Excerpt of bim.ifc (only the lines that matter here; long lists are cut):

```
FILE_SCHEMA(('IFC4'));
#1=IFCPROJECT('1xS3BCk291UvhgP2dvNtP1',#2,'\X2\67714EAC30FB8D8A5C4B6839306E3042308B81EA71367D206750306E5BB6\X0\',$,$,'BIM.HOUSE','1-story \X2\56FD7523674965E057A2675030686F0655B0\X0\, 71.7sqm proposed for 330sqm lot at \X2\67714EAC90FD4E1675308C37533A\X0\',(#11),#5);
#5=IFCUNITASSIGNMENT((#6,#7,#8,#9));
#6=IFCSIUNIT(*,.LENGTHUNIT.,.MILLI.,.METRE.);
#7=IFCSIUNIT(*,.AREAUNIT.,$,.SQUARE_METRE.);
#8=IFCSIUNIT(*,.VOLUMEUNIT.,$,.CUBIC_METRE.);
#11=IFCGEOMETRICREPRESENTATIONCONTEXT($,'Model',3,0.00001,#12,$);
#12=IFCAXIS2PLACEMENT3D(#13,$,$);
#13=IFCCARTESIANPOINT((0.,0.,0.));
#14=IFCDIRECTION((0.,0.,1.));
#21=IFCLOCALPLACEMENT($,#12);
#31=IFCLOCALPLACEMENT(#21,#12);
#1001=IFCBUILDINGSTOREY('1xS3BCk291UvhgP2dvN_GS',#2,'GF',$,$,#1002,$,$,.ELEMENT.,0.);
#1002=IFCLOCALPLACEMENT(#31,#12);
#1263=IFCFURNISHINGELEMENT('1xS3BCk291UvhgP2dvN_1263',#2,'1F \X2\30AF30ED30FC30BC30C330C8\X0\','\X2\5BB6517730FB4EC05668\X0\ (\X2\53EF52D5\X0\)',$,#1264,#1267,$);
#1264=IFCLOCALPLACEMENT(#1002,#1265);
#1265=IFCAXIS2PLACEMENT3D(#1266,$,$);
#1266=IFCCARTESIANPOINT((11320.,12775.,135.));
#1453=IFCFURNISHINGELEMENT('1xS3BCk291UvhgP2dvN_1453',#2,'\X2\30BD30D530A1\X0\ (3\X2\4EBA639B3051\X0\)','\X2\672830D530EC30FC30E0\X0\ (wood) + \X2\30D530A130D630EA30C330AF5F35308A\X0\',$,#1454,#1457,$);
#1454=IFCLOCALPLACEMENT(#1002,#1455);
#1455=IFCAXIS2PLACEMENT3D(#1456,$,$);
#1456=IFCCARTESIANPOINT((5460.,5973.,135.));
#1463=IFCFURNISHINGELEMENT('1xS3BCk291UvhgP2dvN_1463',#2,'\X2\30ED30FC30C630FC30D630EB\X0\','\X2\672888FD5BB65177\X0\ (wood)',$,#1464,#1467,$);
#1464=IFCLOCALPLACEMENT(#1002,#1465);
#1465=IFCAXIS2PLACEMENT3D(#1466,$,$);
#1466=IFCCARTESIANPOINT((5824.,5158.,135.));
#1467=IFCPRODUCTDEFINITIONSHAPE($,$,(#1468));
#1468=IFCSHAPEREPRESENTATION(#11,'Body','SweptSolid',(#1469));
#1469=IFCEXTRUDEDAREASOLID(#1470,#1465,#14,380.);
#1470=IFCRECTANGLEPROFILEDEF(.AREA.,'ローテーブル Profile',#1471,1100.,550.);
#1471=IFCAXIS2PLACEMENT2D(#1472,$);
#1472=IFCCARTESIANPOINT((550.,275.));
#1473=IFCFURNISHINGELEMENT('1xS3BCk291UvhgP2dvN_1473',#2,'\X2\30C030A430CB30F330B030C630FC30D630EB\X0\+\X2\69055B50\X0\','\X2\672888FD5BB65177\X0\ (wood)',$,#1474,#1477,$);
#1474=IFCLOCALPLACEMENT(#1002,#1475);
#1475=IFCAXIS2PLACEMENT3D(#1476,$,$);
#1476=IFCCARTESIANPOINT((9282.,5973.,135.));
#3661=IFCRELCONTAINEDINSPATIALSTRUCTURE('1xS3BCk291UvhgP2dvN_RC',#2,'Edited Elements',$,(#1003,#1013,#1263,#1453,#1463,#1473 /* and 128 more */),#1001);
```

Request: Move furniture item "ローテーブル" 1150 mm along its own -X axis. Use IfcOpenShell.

```python
import ifcopenshell
import ifcopenshell.api.geometry
import ifcopenshell.util.placement
import ifcopenshell.util.unit

model = ifcopenshell.open("bim.ifc")
unit_scale = ifcopenshell.util.unit.calculate_unit_scale(model)

item = model.by_id(1463)
matrix = ifcopenshell.util.placement.get_local_placement(item.ObjectPlacement)
matrix[:3, 3] -= matrix[:3, 0] * 1.15 / unit_scale
ifcopenshell.api.geometry.edit_object_placement(model, product=item, matrix=matrix, is_si=False)

print(ifcopenshell.util.placement.get_local_placement(item.ObjectPlacement).round(3) + 0.0)

model.write("bim_v2.ifc")
```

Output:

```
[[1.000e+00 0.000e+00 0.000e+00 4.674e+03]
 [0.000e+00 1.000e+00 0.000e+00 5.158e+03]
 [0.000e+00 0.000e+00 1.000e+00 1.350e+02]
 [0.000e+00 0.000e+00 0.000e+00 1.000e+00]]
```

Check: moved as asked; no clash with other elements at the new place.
